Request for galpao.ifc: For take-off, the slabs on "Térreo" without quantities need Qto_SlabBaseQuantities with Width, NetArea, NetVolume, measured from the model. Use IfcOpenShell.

First a look at what the model holds.

```python
import ifcopenshell
import ifcopenshell.util.element
import ifcopenshell.util.unit

model = ifcopenshell.open("galpao.ifc")
print(model.schema)
for unit_type in ("LENGTHUNIT", "AREAUNIT", "VOLUMEUNIT"):
    print(unit_type, ifcopenshell.util.unit.calculate_unit_scale(model, unit_type))
storey = next(s for s in model.by_type("IfcBuildingStorey") if s.Name == "Térreo")
slabs = [e for e in ifcopenshell.util.element.get_decomposition(storey) if e.is_a("IfcSlab")]
for e in sorted(slabs, key=lambda e: e.id()):
    print(e.id(), e.is_a(), e.Name, list(ifcopenshell.util.element.get_psets(e, qtos_only=True)), sep=" | ")
```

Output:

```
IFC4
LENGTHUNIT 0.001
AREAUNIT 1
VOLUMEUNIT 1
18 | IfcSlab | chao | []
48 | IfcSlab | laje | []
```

```python
import ifcopenshell
import ifcopenshell.api.pset
import ifcopenshell.geom
import ifcopenshell.util.element
import ifcopenshell.util.shape
import ifcopenshell.util.unit

model = ifcopenshell.open("galpao.ifc")
unit_scale = ifcopenshell.util.unit.calculate_unit_scale(model)
area_scale = ifcopenshell.util.unit.calculate_unit_scale(model, "AREAUNIT")
volume_scale = ifcopenshell.util.unit.calculate_unit_scale(model, "VOLUMEUNIT")
settings = ifcopenshell.geom.settings()

storey = next(s for s in model.by_type("IfcBuildingStorey") if s.Name == "Térreo")
slabs = [e for e in ifcopenshell.util.element.get_decomposition(storey) if e.is_a("IfcSlab")]

for e in sorted(slabs, key=lambda e: e.id()):
    if ifcopenshell.util.element.get_psets(e, qtos_only=True, should_inherit=False):
        continue
    # Geometry comes back in metres, in the element's own axes.
    shape = ifcopenshell.geom.create_shape(settings, e)
    values = {
        "Width": ifcopenshell.util.shape.get_z(shape.geometry) / unit_scale,
        "NetArea": ifcopenshell.util.shape.get_footprint_area(shape.geometry) / area_scale,
        "NetVolume": ifcopenshell.util.shape.get_volume(shape.geometry) / volume_scale,
    }
    qto = ifcopenshell.api.pset.add_qto(model, product=e, name="Qto_SlabBaseQuantities")
    ifcopenshell.api.pset.edit_qto(model, qto=qto, properties=values)
    print(e.id(), {k: round(v, 3) for k, v in values.items()})

model.write("galpao_edited.ifc")
```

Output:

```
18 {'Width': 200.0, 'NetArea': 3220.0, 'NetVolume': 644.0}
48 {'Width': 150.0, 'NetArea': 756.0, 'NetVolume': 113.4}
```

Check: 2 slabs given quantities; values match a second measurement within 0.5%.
